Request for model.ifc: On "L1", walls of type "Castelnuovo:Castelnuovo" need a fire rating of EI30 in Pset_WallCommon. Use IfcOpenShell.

First a look at what the model holds.

```python
import ifcopenshell
import ifcopenshell.util.element

model = ifcopenshell.open("model.ifc")
print(model.schema)
storey = next(s for s in model.by_type("IfcBuildingStorey") if s.Name == "L1")
walls = [e for e in ifcopenshell.util.element.get_decomposition(storey) if e.is_a("IfcWall")]
seen = {}
for e in walls:
    element_type = ifcopenshell.util.element.get_type(e)
    key = (element_type.Name if element_type != e and element_type else None, ifcopenshell.util.element.get_pset(e, "Pset_WallCommon", "FireRating"))
    seen[key] = seen.get(key, 0) + 1
for (name, value), count in sorted(seen.items(), key=str):
    print(count, "x", name, "|", value)
```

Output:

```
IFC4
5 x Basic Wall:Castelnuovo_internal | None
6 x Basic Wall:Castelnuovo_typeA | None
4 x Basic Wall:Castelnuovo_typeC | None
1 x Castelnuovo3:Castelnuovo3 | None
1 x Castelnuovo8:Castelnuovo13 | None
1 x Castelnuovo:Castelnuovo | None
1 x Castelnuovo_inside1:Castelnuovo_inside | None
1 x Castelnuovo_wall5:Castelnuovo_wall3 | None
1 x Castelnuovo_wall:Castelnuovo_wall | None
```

```python
import ifcopenshell
import ifcopenshell.api.pset
import ifcopenshell.util.element

model = ifcopenshell.open("model.ifc")

storey = next(s for s in model.by_type("IfcBuildingStorey") if s.Name == "L1")
walls = [e for e in ifcopenshell.util.element.get_decomposition(storey) if e.is_a("IfcWall")]

count = 0
for e in walls:
    element_type = ifcopenshell.util.element.get_type(e)
    if element_type in (None, e) or element_type.Name != "Castelnuovo:Castelnuovo":
        continue
    # add_pset returns the element's existing set when there is one.
    pset = ifcopenshell.api.pset.add_pset(model, product=e, name="Pset_WallCommon")
    ifcopenshell.api.pset.edit_pset(model, pset=pset, properties={"FireRating": "EI30"})
    count += 1

print(count, "walls updated")

model.write("model_edited.ifc")
```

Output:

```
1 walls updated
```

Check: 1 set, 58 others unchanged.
